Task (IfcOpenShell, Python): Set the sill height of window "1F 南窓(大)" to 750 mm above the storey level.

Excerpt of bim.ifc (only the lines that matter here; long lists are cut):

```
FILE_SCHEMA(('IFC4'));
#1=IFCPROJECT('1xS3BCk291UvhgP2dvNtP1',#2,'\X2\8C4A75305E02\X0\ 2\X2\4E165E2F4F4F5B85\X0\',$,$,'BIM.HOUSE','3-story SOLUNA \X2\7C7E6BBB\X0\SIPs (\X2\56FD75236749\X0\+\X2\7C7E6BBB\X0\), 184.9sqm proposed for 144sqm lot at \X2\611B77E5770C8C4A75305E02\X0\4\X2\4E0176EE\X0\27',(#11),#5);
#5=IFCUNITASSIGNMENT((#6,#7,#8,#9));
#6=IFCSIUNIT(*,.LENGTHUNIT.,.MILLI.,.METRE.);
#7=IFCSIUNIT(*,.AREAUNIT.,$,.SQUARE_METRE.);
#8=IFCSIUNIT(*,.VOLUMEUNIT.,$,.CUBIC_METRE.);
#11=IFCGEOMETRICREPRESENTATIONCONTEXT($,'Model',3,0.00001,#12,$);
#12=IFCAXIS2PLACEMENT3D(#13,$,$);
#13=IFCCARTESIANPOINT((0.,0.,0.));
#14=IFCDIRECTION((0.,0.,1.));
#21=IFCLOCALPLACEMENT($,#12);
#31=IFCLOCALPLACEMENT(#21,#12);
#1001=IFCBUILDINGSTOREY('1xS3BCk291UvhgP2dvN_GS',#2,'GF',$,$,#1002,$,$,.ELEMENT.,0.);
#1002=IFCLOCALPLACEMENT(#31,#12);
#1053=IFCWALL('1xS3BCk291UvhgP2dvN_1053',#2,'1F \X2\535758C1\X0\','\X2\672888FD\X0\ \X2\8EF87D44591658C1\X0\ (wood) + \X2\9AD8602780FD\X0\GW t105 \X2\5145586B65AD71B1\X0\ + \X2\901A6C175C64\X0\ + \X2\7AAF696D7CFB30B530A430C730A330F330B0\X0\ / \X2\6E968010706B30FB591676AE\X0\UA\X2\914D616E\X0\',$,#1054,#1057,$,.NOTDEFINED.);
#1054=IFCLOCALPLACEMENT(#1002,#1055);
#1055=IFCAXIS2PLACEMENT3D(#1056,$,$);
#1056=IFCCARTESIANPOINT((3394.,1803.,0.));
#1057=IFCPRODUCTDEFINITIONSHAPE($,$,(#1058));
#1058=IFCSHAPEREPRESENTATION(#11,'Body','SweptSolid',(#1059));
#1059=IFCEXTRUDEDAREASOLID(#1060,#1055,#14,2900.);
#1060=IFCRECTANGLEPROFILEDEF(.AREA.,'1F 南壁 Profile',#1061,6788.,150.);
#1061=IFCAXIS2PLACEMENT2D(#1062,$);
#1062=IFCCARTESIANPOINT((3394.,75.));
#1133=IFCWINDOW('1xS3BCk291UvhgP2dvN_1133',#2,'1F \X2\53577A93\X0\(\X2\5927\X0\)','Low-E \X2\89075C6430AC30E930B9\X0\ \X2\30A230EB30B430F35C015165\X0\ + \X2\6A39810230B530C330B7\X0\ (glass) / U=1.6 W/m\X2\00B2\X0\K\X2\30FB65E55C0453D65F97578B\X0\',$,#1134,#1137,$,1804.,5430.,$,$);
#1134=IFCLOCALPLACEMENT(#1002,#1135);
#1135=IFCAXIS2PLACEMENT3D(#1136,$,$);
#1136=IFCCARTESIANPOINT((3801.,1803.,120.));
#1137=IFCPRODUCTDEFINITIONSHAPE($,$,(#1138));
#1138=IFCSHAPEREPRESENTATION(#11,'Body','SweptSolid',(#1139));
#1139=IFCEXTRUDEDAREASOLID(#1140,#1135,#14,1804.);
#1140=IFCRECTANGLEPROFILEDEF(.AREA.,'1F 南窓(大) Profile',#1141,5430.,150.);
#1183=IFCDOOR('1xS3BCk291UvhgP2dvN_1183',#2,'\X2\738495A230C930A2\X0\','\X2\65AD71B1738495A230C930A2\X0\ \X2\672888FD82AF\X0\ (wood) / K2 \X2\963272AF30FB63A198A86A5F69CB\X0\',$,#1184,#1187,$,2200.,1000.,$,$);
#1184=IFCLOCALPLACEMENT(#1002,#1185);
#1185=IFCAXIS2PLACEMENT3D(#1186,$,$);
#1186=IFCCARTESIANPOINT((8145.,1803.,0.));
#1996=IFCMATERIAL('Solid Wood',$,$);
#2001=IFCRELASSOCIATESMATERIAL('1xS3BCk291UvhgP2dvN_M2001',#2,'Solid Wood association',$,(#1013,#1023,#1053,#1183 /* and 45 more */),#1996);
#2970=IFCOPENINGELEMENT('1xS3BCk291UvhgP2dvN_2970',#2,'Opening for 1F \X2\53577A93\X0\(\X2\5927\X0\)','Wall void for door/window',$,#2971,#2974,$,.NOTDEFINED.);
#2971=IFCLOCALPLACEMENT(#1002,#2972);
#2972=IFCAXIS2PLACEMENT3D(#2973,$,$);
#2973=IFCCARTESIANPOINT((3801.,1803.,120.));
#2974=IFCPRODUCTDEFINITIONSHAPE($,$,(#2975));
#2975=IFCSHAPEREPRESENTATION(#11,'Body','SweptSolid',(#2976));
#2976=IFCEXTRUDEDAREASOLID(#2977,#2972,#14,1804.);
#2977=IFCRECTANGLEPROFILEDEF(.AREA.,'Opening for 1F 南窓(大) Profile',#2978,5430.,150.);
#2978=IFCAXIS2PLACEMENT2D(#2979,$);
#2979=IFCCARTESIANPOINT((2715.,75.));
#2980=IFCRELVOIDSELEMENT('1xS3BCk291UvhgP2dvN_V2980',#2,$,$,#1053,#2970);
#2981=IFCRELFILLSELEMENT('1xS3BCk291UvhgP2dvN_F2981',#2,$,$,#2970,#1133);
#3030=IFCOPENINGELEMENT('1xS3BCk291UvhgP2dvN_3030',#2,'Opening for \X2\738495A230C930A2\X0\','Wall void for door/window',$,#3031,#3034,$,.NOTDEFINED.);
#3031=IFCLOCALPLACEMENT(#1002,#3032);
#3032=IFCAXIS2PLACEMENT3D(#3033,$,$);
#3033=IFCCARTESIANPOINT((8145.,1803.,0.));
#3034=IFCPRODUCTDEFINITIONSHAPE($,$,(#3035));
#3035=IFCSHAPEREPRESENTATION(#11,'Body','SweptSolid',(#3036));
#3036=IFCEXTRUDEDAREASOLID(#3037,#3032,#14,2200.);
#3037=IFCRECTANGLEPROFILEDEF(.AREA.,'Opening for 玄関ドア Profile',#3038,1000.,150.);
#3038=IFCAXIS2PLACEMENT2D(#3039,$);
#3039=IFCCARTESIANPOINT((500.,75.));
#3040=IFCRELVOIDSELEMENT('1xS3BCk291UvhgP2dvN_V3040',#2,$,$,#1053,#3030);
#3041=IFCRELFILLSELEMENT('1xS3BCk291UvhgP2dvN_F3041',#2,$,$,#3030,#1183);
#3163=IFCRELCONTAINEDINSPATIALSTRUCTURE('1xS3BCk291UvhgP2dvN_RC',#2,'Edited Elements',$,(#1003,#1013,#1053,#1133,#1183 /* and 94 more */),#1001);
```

```python
import numpy as np
import ifcopenshell
import ifcopenshell.api.geometry
import ifcopenshell.geom
import ifcopenshell.util.element
import ifcopenshell.util.placement
import ifcopenshell.util.shape
import ifcopenshell.util.unit

model = ifcopenshell.open("bim.ifc")
unit_scale = ifcopenshell.util.unit.calculate_unit_scale(model)

window = model.by_guid("1xS3BCk291UvhgP2dvN_1133")
opening = window.FillsVoids[0].RelatingOpeningElement
storey = ifcopenshell.util.element.get_container(window, ifc_class="IfcBuildingStorey")
level = ifcopenshell.util.placement.get_local_placement(storey.ObjectPlacement)[2, 3]

# The opening's origin need not be at the sill, so measure its lowest point.
shape = ifcopenshell.geom.create_shape(ifcopenshell.geom.settings(), opening)
bottom = ifcopenshell.util.shape.get_shape_bottom_elevation(shape, shape.geometry) / unit_scale
dz = level + 0.75 / unit_scale - bottom

shift = np.array([0.0, 0.0, dz])
# The window is not placed relative to its opening, so move both.
for product in (opening, window):
    matrix = ifcopenshell.util.placement.get_local_placement(product.ObjectPlacement)
    matrix[:3, 3] += shift
    ifcopenshell.api.geometry.edit_object_placement(model, product=product, matrix=matrix, is_si=False)

print(f"moved by {dz * unit_scale:+.3f} m")

model.write("bim_rev.ifc")
```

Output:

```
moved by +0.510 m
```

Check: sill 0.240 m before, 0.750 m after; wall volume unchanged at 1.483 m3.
